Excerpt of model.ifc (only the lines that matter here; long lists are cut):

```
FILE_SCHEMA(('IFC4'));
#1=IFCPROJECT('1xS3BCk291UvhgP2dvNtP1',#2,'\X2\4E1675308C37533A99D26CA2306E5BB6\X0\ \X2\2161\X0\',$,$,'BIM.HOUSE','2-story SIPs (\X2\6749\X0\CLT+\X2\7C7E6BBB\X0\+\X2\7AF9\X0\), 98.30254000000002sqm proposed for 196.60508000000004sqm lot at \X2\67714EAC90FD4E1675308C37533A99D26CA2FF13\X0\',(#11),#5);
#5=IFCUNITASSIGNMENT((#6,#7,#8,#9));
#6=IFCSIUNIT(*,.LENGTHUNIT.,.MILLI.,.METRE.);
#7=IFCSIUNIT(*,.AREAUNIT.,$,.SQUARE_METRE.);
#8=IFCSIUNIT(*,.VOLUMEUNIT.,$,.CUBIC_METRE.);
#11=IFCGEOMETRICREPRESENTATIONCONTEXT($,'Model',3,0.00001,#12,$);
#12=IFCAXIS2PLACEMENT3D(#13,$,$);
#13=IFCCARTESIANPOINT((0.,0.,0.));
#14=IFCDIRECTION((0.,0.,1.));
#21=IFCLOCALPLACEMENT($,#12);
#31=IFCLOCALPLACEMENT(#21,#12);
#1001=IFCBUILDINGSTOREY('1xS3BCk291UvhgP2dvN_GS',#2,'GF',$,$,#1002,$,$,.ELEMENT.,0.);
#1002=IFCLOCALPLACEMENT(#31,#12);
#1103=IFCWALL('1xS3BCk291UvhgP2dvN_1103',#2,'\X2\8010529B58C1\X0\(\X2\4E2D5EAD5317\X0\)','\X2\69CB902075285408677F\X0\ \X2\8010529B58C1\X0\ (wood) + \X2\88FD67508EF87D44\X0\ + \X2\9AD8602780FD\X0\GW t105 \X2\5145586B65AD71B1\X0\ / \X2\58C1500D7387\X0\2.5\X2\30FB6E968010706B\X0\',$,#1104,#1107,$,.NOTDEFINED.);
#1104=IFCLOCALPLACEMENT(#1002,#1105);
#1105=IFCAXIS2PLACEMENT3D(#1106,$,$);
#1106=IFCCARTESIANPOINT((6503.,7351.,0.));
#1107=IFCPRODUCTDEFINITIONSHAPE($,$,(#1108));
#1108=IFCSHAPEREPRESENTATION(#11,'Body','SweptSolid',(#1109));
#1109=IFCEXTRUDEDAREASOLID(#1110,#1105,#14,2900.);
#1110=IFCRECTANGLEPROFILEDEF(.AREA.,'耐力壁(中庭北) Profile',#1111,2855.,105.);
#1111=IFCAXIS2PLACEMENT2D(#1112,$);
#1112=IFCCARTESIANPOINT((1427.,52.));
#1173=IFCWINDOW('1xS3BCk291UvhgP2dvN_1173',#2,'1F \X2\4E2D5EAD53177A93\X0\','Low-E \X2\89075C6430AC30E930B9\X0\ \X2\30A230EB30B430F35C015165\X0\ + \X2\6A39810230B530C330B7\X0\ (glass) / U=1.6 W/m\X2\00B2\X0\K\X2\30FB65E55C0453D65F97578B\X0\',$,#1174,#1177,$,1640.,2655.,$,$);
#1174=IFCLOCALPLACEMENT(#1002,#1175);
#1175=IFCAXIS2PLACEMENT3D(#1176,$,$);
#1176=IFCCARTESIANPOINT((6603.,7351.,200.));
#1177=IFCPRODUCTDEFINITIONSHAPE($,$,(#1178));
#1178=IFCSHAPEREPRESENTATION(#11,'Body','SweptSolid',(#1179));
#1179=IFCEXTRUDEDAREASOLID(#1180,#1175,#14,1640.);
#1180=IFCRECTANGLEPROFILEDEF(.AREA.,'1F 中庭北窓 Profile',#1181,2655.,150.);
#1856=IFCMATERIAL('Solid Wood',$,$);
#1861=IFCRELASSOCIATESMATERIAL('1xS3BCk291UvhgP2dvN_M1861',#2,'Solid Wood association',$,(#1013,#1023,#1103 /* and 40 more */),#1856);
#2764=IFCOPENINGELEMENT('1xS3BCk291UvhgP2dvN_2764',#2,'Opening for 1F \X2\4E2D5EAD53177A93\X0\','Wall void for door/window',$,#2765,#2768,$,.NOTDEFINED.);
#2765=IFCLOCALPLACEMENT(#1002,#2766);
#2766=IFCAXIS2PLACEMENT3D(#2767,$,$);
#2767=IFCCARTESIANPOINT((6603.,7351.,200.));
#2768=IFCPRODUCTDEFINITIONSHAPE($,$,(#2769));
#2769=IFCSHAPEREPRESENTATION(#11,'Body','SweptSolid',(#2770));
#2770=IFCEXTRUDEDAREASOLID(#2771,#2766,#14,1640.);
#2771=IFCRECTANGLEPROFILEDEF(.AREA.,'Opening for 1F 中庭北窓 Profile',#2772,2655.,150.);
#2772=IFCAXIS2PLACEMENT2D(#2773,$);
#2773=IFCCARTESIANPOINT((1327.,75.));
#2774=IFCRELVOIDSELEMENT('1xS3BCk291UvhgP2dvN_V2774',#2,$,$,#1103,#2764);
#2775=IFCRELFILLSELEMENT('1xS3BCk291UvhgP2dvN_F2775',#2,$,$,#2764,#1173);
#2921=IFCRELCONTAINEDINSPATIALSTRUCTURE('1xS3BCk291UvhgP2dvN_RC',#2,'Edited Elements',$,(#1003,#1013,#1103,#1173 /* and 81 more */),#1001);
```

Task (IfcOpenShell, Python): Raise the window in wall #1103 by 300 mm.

```python
import numpy as np
import ifcopenshell
import ifcopenshell.api.geometry
import ifcopenshell.util.placement
import ifcopenshell.util.unit

model = ifcopenshell.open("model.ifc")
unit_scale = ifcopenshell.util.unit.calculate_unit_scale(model)

window = model.by_guid("1xS3BCk291UvhgP2dvN_1173")
opening = window.FillsVoids[0].RelatingOpeningElement
dz = 0.3 / unit_scale

shift = np.array([0.0, 0.0, dz])
# The window is not placed relative to its opening, so move both.
for product in (opening, window):
    matrix = ifcopenshell.util.placement.get_local_placement(product.ObjectPlacement)
    matrix[:3, 3] += shift
    ifcopenshell.api.geometry.edit_object_placement(model, product=product, matrix=matrix, is_si=False)

print(f"moved by {dz * unit_scale:+.3f} m")

model.write("model_updated.ifc")
```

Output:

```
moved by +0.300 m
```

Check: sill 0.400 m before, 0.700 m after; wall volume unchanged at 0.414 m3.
